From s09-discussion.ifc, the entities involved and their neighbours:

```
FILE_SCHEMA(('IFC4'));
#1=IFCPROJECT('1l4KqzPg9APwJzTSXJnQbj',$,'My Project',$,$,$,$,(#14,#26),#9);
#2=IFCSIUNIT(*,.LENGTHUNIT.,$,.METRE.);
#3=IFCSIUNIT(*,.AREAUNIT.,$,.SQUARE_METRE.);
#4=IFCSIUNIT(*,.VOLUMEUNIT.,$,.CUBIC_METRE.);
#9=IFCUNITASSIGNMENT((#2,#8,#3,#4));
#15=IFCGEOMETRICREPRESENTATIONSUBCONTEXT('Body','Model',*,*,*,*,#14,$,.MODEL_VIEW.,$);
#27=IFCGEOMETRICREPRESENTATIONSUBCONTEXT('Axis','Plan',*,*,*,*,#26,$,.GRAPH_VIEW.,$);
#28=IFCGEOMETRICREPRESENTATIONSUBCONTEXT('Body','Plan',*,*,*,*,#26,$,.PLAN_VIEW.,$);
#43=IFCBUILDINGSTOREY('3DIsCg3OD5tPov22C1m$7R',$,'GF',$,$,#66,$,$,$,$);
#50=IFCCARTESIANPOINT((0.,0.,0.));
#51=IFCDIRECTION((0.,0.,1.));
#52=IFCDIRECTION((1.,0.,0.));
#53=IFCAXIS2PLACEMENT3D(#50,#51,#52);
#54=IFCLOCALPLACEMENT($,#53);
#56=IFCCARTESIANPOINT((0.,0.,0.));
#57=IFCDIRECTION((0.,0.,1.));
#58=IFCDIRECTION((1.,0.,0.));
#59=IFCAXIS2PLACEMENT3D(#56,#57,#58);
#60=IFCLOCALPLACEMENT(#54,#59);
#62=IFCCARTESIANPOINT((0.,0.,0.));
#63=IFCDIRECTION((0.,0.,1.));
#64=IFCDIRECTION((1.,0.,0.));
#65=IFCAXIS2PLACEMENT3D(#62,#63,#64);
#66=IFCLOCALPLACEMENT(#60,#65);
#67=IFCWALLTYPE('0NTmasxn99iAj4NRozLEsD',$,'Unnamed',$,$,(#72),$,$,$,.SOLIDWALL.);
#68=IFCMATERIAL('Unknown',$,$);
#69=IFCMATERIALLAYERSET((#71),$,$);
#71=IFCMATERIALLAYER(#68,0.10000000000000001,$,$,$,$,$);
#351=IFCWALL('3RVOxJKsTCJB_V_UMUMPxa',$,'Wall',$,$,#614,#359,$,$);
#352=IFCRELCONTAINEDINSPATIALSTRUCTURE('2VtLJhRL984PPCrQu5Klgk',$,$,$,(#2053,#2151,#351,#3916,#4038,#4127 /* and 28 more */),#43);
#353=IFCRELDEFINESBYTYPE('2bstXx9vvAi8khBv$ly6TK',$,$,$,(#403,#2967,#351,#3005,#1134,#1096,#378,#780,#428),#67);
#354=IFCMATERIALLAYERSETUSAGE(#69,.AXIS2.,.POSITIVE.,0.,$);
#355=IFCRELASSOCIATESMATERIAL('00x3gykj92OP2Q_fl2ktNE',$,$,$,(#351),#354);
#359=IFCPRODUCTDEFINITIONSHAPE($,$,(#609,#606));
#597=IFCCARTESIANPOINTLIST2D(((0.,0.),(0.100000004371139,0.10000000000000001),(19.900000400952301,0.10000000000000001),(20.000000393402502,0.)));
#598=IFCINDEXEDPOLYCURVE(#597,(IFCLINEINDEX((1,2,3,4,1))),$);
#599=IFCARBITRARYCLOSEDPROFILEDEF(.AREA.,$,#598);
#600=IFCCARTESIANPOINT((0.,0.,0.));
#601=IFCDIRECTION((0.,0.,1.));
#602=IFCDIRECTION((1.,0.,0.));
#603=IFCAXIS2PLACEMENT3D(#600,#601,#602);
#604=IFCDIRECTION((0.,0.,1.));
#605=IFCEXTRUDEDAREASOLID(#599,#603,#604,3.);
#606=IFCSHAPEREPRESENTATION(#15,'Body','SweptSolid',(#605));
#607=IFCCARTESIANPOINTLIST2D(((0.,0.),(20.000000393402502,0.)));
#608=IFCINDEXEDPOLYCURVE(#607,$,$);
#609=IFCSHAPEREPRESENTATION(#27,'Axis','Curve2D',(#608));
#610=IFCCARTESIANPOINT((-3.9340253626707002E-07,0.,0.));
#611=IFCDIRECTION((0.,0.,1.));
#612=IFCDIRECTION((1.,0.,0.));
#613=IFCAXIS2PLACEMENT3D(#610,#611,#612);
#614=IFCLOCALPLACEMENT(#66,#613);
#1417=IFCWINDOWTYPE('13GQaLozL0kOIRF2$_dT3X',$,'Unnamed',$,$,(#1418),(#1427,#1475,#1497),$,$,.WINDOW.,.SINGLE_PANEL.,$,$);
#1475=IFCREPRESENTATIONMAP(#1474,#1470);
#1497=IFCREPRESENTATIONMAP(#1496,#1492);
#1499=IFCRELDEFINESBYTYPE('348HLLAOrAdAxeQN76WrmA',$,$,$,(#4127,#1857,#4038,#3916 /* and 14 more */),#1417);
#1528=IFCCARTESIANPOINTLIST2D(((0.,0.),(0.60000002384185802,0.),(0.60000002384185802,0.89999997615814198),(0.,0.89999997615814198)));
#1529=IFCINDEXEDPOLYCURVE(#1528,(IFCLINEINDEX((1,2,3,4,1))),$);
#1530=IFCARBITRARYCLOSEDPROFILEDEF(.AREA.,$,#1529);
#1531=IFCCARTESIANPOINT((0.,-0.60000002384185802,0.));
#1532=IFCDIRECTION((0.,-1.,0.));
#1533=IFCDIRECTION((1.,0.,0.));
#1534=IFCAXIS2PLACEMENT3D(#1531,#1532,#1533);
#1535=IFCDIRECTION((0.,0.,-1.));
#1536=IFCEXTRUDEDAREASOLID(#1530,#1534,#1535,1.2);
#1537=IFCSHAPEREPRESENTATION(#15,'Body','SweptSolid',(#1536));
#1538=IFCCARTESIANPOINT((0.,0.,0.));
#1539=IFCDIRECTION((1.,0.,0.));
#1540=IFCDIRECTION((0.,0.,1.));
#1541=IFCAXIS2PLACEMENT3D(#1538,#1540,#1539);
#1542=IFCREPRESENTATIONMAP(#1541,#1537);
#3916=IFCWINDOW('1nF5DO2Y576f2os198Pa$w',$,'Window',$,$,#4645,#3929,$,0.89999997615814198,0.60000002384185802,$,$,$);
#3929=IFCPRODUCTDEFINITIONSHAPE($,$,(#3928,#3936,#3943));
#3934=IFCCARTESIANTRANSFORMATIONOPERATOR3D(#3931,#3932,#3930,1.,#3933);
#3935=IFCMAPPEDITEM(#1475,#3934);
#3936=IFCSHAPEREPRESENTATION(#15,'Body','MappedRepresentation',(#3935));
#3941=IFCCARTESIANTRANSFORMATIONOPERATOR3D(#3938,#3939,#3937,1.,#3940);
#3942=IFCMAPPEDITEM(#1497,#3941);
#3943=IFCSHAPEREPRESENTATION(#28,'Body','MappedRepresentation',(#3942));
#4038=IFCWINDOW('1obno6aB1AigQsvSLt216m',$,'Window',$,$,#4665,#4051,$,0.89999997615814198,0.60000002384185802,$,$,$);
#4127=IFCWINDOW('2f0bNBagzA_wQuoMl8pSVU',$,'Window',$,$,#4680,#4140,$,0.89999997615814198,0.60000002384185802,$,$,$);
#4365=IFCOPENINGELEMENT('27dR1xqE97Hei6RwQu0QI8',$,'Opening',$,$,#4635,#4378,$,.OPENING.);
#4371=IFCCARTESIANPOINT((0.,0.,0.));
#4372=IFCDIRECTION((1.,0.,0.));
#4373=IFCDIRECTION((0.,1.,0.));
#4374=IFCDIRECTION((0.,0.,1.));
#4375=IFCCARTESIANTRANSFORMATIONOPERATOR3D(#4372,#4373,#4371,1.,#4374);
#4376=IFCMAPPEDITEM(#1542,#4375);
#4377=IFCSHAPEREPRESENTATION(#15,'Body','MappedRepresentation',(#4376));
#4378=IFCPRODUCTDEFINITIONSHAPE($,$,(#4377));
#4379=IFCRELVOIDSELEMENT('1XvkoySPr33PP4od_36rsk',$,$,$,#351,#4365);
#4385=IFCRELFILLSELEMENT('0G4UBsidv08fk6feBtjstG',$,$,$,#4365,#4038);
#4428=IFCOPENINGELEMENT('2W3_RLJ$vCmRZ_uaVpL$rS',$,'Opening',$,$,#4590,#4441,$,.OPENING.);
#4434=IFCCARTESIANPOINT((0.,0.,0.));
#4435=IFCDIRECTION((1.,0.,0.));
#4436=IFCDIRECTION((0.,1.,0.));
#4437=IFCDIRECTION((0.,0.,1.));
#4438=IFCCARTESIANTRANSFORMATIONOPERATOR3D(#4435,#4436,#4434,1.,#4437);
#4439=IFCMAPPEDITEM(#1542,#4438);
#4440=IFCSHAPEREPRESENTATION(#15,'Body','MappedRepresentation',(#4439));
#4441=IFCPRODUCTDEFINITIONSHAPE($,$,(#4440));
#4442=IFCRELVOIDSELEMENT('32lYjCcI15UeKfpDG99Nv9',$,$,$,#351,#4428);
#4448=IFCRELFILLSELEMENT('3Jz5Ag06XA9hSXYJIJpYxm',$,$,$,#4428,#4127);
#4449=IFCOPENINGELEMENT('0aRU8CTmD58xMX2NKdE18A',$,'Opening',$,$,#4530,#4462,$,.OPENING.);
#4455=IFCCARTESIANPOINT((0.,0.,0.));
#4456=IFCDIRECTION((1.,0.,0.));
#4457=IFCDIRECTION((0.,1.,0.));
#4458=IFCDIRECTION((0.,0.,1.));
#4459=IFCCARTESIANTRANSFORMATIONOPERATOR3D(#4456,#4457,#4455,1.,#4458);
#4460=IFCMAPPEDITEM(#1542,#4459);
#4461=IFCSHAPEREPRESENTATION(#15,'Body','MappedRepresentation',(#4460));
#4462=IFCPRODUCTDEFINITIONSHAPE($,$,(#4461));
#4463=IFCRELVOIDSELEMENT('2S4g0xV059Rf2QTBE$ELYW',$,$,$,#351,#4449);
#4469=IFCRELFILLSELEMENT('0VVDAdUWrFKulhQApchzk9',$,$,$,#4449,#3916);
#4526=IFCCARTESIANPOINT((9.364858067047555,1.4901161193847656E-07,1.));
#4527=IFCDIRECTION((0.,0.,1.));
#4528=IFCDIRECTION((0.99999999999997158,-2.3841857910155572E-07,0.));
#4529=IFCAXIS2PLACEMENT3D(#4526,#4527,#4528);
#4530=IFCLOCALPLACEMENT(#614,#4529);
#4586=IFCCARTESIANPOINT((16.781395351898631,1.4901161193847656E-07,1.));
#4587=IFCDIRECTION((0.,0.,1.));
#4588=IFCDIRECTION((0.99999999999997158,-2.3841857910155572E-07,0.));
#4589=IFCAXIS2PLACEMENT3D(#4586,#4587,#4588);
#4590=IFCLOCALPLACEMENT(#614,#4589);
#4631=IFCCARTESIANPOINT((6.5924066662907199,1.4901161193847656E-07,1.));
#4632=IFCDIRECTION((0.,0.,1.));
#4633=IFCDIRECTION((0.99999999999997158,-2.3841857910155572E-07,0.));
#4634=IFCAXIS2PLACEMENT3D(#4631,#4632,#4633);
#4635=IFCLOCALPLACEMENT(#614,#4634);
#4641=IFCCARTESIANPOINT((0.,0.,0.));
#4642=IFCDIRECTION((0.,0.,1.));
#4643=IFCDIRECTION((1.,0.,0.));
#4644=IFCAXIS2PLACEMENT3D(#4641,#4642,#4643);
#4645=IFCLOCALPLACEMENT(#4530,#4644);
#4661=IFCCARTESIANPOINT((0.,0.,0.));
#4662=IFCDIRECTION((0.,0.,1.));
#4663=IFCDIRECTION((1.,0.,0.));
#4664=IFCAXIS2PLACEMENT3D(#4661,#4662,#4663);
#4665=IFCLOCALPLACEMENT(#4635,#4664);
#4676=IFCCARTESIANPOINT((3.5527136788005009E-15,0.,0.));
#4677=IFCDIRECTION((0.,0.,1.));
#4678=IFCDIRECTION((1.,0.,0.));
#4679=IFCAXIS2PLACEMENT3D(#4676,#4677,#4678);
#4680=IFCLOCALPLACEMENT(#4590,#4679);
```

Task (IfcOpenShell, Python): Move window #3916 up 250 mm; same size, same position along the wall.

```python
import numpy as np
import ifcopenshell
import ifcopenshell.api.geometry
import ifcopenshell.util.placement
import ifcopenshell.util.unit

model = ifcopenshell.open("s09-discussion.ifc")
unit_scale = ifcopenshell.util.unit.calculate_unit_scale(model)

window = model.by_guid("1nF5DO2Y576f2os198Pa$w")
opening = window.FillsVoids[0].RelatingOpeningElement
dz = 0.25

shift = np.array([0.0, 0.0, dz])
# The window is placed relative to its opening, so it follows when the opening moves.
matrix = ifcopenshell.util.placement.get_local_placement(opening.ObjectPlacement)
matrix[:3, 3] += shift
ifcopenshell.api.geometry.edit_object_placement(
    model, product=opening, matrix=matrix, is_si=False, should_transform_children=True
)

print(f"moved by {dz * unit_scale:+.3f} m")

model.write("s09-discussion_rev.ifc")
```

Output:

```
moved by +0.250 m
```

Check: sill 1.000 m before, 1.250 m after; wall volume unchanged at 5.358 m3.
